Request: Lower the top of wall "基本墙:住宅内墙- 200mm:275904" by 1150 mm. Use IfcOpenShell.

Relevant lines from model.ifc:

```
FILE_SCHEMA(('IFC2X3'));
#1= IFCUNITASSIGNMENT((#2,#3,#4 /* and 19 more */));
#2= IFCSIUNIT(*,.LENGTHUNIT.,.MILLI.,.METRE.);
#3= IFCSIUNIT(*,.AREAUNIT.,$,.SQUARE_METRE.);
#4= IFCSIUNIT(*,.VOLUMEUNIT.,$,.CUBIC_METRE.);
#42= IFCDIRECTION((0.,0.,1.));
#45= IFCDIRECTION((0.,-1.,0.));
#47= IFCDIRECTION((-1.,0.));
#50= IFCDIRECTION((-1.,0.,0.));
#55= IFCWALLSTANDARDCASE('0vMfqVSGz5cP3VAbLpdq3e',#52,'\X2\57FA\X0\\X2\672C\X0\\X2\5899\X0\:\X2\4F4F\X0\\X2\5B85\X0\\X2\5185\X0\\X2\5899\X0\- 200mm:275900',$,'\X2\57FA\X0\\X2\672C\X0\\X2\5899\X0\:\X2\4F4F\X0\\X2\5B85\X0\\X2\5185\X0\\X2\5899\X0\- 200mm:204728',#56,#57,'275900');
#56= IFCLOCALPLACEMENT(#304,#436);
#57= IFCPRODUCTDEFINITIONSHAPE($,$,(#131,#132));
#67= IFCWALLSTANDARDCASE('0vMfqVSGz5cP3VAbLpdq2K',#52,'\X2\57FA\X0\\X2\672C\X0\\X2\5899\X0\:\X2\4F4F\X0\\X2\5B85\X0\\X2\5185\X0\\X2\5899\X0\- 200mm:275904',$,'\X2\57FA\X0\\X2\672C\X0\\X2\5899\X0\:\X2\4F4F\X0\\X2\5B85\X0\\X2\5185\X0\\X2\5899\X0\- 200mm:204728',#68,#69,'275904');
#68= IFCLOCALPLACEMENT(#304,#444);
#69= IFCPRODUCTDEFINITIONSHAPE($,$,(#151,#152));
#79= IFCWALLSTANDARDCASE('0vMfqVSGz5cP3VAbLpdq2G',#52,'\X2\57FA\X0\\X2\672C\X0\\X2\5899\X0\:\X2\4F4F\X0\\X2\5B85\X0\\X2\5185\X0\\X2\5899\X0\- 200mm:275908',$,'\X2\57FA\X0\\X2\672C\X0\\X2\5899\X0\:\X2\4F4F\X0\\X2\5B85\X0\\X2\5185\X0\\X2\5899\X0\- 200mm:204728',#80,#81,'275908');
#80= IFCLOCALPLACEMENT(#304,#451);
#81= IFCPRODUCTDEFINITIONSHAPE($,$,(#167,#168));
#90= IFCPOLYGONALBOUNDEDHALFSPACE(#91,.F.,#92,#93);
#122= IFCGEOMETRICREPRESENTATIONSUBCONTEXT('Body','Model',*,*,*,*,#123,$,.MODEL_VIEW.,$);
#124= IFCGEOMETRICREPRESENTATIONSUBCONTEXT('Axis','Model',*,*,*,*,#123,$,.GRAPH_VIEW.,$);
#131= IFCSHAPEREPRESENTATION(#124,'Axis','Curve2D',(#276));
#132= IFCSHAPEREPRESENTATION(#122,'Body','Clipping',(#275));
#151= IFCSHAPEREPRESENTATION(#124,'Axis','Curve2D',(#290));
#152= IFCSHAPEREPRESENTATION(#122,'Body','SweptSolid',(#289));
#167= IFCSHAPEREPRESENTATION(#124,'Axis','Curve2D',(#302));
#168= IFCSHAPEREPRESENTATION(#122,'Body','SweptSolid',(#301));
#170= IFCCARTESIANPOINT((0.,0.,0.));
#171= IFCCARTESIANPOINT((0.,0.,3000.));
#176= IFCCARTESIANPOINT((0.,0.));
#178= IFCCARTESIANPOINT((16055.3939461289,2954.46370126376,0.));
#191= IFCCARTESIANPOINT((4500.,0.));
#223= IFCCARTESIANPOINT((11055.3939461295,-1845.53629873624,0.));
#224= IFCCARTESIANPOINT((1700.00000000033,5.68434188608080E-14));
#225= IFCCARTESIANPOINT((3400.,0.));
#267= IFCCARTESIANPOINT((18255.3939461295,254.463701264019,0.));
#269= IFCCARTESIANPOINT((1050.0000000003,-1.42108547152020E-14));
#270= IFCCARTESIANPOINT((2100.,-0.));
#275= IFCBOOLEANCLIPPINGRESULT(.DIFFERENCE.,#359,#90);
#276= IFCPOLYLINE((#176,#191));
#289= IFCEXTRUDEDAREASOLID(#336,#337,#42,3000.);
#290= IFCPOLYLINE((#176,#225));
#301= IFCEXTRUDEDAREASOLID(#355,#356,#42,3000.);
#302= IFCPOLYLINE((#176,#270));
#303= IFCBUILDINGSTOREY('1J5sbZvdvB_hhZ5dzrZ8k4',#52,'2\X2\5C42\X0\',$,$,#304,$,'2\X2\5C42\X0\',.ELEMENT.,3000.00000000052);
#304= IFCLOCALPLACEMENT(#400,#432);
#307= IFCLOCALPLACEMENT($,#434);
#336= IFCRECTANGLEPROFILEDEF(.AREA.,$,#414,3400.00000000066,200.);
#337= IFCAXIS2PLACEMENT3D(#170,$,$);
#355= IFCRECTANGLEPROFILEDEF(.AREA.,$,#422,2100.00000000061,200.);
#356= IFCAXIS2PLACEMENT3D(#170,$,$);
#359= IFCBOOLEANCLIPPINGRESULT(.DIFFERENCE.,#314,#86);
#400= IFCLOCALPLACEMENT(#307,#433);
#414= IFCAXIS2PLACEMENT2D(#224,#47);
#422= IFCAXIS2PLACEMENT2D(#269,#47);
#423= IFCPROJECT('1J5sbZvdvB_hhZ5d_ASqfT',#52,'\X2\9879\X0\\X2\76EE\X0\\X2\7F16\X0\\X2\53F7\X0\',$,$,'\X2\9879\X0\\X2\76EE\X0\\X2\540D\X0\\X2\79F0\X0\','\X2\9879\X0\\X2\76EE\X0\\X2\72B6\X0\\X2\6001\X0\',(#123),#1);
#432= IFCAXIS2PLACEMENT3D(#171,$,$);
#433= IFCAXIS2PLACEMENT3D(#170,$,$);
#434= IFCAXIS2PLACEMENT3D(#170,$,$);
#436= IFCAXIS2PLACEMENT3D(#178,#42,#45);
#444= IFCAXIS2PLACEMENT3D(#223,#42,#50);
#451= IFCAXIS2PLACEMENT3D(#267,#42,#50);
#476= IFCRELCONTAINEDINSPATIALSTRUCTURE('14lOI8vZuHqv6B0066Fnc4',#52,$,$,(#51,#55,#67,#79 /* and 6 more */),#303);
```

```python
import ifcopenshell
import ifcopenshell.geom
import ifcopenshell.util.representation
import ifcopenshell.util.shape

model = ifcopenshell.open("model.ifc")
settings = ifcopenshell.geom.settings()


def volume(element):
    """Net volume in cubic metres, openings subtracted."""
    shape = ifcopenshell.geom.create_shape(settings, element)
    return ifcopenshell.util.shape.get_volume(shape.geometry)


wall = model.by_id(67)
before = volume(wall)

body = ifcopenshell.util.representation.get_representation(wall, "Model", "Body")
solid = body.Items[0]
old_height = solid.Depth
solid.Depth -= 1150.0
after = volume(wall)

print(f"height {old_height:g} -> {solid.Depth:g}, volume {before:.3f} -> {after:.3f} m3")

model.write("model_updated.ifc")
```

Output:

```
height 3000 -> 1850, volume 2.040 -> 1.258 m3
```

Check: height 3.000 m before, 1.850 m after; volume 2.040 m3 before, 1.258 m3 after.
